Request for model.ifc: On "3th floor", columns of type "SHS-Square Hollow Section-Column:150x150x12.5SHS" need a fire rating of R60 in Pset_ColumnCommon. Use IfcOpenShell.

First a look at what the model holds.

```python
import ifcopenshell
import ifcopenshell.util.element

model = ifcopenshell.open("model.ifc")
print(model.schema)
storey = next(s for s in model.by_type("IfcBuildingStorey") if s.Name == "3th floor")
columns = [e for e in ifcopenshell.util.element.get_decomposition(storey) if e.is_a("IfcColumn")]
seen = {}
for e in columns:
    element_type = ifcopenshell.util.element.get_type(e)
    key = (element_type.Name if element_type != e and element_type else None, ifcopenshell.util.element.get_pset(e, "Pset_ColumnCommon", "FireRating"))
    seen[key] = seen.get(key, 0) + 1
for (name, value), count in sorted(seen.items(), key=str):
    print(count, "x", name, "|", value)
```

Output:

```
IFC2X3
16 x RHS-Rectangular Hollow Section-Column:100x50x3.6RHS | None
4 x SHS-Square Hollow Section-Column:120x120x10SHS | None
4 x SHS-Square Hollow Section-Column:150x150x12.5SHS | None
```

```python
import ifcopenshell
import ifcopenshell.api.pset
import ifcopenshell.util.element

model = ifcopenshell.open("model.ifc")

storey = next(s for s in model.by_type("IfcBuildingStorey") if s.Name == "3th floor")
columns = [e for e in ifcopenshell.util.element.get_decomposition(storey) if e.is_a("IfcColumn")]

count = 0
for e in columns:
    element_type = ifcopenshell.util.element.get_type(e)
    if element_type in (None, e) or element_type.Name != "SHS-Square Hollow Section-Column:150x150x12.5SHS":
        continue
    # add_pset returns the element's existing set when there is one.
    pset = ifcopenshell.api.pset.add_pset(model, product=e, name="Pset_ColumnCommon")
    ifcopenshell.api.pset.edit_pset(model, pset=pset, properties={"FireRating": "R60"})
    count += 1

print(count, "columns updated")

model.write("model_rev.ifc")
```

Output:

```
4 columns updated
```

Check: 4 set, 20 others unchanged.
